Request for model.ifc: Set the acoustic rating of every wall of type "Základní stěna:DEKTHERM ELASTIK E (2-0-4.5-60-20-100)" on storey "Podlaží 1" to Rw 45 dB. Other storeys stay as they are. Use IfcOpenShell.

First a look at what the model holds.

```python
import ifcopenshell
import ifcopenshell.util.element

model = ifcopenshell.open("model.ifc")
print(model.schema)
storey = next(s for s in model.by_type("IfcBuildingStorey") if s.Name == "Podlaží 1")
walls = [e for e in ifcopenshell.util.element.get_decomposition(storey) if e.is_a("IfcWall")]
seen = {}
for e in walls:
    element_type = ifcopenshell.util.element.get_type(e)
    key = (element_type.Name if element_type != e and element_type else None, ifcopenshell.util.element.get_pset(e, "Pset_WallCommon", "AcousticRating"))
    seen[key] = seen.get(key, 0) + 1
for (name, value), count in sorted(seen.items(), key=str):
    print(count, "x", name, "|", value)
```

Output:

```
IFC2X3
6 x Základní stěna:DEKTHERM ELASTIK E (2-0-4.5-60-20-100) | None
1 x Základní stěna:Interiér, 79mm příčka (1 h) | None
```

```python
import ifcopenshell
import ifcopenshell.api.pset
import ifcopenshell.util.element

model = ifcopenshell.open("model.ifc")

storey = next(s for s in model.by_type("IfcBuildingStorey") if s.Name == "Podlaží 1")
walls = [e for e in ifcopenshell.util.element.get_decomposition(storey) if e.is_a("IfcWall")]

count = 0
for e in walls:
    element_type = ifcopenshell.util.element.get_type(e)
    if element_type in (None, e) or element_type.Name != "Základní stěna:DEKTHERM ELASTIK E (2-0-4.5-60-20-100)":
        continue
    # add_pset returns the element's existing set when there is one.
    pset = ifcopenshell.api.pset.add_pset(model, product=e, name="Pset_WallCommon")
    ifcopenshell.api.pset.edit_pset(model, pset=pset, properties={"AcousticRating": "Rw 45 dB"})
    count += 1

print(count, "walls updated")

model.write("model_edited.ifc")
```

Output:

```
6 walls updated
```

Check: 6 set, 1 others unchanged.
